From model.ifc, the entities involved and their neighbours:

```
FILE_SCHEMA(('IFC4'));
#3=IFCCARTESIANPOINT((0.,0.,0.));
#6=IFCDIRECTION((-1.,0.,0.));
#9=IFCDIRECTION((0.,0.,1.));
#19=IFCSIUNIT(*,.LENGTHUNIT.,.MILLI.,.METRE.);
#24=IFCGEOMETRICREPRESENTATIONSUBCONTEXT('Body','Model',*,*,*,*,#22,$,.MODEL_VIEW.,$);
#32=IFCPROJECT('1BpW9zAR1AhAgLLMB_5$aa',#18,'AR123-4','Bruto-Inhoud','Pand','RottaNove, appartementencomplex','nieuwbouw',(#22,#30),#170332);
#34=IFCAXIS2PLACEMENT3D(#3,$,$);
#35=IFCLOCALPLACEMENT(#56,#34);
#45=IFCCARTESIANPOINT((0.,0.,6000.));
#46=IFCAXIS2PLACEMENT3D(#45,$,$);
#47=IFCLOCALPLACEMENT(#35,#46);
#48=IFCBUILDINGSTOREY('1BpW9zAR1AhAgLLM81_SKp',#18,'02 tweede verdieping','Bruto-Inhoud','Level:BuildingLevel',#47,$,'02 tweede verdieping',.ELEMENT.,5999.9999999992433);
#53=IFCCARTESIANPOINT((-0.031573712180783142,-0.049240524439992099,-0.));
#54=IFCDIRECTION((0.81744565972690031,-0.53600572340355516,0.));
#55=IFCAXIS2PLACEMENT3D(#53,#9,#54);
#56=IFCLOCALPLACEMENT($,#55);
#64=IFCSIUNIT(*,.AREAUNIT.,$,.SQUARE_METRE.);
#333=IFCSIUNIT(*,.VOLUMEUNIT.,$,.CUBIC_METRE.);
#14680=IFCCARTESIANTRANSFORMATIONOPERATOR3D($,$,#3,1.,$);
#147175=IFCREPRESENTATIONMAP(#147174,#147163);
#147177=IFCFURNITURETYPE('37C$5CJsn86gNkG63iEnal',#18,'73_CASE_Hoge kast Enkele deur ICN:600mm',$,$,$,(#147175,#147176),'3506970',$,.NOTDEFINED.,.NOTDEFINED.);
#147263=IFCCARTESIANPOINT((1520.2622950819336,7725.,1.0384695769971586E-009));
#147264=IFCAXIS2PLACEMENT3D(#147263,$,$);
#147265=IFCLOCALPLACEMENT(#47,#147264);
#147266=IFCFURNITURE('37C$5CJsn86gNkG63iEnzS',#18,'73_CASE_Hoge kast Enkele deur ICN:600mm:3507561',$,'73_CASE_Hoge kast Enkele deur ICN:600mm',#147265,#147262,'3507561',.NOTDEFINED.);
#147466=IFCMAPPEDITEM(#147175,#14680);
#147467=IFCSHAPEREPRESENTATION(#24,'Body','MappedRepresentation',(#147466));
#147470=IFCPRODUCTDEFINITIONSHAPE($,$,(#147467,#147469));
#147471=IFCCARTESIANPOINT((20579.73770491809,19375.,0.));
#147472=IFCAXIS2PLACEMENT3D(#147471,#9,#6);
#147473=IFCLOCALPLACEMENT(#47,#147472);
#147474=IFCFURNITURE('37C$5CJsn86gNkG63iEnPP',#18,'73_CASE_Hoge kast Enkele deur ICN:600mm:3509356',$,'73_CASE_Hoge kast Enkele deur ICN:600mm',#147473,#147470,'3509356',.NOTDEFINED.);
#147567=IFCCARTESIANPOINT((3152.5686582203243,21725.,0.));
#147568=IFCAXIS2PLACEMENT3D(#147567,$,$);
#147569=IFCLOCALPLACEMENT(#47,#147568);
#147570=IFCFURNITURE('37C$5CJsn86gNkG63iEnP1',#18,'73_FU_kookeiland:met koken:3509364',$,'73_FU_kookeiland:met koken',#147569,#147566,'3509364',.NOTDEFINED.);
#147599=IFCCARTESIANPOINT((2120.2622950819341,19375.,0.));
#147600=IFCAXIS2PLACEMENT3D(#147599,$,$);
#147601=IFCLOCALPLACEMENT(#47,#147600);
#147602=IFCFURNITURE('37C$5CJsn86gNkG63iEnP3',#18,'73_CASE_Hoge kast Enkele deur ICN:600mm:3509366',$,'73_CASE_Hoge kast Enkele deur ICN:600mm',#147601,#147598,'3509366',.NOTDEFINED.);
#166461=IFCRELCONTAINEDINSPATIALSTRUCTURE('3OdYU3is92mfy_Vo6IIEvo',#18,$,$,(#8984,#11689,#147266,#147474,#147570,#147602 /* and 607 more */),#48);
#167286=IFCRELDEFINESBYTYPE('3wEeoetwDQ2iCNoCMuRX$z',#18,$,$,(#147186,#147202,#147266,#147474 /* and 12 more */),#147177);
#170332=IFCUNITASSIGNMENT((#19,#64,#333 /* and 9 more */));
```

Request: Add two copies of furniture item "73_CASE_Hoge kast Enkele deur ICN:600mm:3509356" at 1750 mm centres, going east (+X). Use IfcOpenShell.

```python
import numpy as np
import ifcopenshell
import ifcopenshell.api.geometry
import ifcopenshell.api.root
import ifcopenshell.util.element
import ifcopenshell.util.placement
import ifcopenshell.util.unit

model = ifcopenshell.open("model.ifc")
unit_scale = ifcopenshell.util.unit.calculate_unit_scale(model)


def reuse_history(source, copy):
    """copy_class also copies each property set's owner history, people and application; keep the originals."""
    for rel in copy.IsDefinedBy:
        if rel.is_a("IfcRelDefinesByProperties") and (history := rel.RelatingPropertyDefinition.OwnerHistory):
            rel.RelatingPropertyDefinition.OwnerHistory = source.OwnerHistory
            ifcopenshell.util.element.remove_deep2(model, history)


source = model.by_guid("37C$5CJsn86gNkG63iEnPP")
base = ifcopenshell.util.placement.get_local_placement(source.ObjectPlacement)
step = np.array([1.0, 0.0, 0.0]) * 1.75 / unit_scale

for i in range(1, 3):
    copy = ifcopenshell.api.root.copy_class(model, product=source)
    copy.Representation = ifcopenshell.util.element.copy_deep(
        model, source.Representation, exclude=["IfcGeometricRepresentationContext", "IfcRepresentationMap"]
    )
    copy.Name = "73_CASE_Hoge kast Enkele deur ICN:600mm"
    copy.Tag = None
    reuse_history(source, copy)
    matrix = base.copy()
    matrix[:3, 3] += i * step
    print("added at", matrix[:3, 3].round(3) + 0.0)
    ifcopenshell.api.geometry.edit_object_placement(model, product=copy, matrix=matrix, is_si=False)

model.write("model-out.ifc")
```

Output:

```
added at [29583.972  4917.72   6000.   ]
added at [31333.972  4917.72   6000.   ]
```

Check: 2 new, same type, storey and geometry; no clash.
